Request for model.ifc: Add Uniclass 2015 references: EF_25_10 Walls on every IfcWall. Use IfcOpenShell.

First a look at what the model holds.

```python
import ifcopenshell

model = ifcopenshell.open("model.ifc")
print(model.schema)
print("classifications:", [c.Name for c in model.by_type("IfcClassification")])
for ifc_class in ("IfcDoor", "IfcRoof", "IfcStair", "IfcWall", "IfcWindow"):
    print(ifc_class, len(model.by_type(ifc_class)))
```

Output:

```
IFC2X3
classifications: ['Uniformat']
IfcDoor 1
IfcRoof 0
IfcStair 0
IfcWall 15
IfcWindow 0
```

```python
import ifcopenshell
import ifcopenshell.api.classification

model = ifcopenshell.open("model.ifc")

# IFC2X3 requires Source and Edition and has no link from the project to the system.
system = model.create_entity("IfcClassification", Source="NBS", Edition="2015", Name="Uniclass 2015")

codes = {
    "IfcWall": ("EF_25_10", "Walls"),
}
for ifc_class, (code, name) in codes.items():
    products = model.by_type(ifc_class)
    ifcopenshell.api.classification.add_reference(
        model, products=products, classification=system, identification=code, name=name
    )
    print(code, len(products))

model.write("model_edited.ifc")
```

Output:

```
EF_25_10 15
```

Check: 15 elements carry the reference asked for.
